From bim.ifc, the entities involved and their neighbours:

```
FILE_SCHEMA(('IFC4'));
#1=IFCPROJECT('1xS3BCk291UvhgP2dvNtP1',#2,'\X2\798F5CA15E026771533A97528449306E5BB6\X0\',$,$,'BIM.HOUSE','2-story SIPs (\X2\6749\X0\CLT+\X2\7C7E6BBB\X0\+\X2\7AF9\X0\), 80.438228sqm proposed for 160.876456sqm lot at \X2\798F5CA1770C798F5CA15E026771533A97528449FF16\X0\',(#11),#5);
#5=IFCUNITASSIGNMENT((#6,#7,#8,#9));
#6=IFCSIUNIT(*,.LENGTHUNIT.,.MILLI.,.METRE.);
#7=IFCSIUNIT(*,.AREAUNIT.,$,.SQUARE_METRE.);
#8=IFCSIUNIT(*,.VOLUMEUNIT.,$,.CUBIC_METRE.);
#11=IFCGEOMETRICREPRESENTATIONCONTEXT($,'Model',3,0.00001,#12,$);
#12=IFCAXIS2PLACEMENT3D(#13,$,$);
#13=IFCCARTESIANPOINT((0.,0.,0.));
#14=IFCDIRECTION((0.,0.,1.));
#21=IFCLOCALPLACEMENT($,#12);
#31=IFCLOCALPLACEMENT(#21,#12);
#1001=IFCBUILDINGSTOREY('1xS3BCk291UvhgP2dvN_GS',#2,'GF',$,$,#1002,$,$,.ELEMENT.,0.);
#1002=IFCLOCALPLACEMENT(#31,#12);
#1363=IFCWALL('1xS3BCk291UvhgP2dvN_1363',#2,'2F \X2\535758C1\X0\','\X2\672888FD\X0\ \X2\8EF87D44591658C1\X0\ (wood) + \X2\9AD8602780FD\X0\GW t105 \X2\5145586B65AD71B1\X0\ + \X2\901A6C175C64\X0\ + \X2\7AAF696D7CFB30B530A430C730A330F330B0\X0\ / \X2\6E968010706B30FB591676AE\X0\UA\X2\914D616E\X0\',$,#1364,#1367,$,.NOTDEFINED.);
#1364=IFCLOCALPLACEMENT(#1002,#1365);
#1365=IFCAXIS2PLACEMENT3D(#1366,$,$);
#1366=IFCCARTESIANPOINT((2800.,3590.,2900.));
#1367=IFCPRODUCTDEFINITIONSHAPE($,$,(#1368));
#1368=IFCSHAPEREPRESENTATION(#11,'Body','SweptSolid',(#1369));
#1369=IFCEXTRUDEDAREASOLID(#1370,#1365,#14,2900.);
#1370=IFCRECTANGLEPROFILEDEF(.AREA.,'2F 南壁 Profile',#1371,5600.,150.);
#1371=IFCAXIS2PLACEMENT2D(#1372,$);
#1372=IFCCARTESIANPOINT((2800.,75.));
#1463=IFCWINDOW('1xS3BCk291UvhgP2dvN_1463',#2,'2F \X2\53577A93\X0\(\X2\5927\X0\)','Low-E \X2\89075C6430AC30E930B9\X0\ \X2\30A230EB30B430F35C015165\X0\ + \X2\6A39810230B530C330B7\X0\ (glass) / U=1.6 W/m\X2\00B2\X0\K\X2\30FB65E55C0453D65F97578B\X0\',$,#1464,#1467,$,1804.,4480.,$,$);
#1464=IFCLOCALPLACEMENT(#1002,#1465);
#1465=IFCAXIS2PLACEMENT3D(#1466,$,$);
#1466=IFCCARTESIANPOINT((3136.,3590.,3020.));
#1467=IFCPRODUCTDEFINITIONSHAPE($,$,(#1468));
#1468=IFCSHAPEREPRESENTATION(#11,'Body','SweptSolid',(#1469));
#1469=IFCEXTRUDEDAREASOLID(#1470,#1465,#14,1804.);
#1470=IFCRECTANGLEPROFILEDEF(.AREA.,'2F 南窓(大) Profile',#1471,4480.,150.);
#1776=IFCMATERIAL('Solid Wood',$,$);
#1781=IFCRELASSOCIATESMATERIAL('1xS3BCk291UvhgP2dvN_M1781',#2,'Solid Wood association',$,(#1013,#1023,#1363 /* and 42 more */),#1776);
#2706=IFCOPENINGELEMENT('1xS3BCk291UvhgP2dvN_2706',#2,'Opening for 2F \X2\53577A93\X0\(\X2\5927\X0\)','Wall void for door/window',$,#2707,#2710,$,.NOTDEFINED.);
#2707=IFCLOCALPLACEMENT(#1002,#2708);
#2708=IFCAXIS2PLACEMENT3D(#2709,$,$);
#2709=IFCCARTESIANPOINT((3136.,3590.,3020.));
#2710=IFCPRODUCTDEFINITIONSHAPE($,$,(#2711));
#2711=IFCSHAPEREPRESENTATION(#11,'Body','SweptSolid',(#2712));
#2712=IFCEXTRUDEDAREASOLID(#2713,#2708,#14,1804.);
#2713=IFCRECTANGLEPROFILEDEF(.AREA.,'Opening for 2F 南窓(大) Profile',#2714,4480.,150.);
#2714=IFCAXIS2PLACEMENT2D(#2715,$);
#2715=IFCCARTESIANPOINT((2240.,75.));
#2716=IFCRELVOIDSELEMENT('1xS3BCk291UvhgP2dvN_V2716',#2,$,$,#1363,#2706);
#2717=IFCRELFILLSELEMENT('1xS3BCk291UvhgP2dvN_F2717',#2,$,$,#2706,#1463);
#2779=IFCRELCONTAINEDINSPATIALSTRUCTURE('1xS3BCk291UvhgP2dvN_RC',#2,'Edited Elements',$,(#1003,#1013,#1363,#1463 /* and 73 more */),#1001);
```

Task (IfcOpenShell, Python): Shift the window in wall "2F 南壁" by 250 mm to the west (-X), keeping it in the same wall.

```python
import ifcopenshell
import ifcopenshell.api.geometry
import ifcopenshell.util.placement
import ifcopenshell.util.unit

model = ifcopenshell.open("bim.ifc")
unit_scale = ifcopenshell.util.unit.calculate_unit_scale(model)

window = model.by_id(1463)
opening = window.FillsVoids[0].RelatingOpeningElement
wall = opening.VoidsElements[0].RelatingBuildingElement

wall_matrix = ifcopenshell.util.placement.get_local_placement(wall.ObjectPlacement)
shift = wall_matrix[:3, 0] * -0.25 / unit_scale
before = ifcopenshell.util.placement.get_local_placement(window.ObjectPlacement)[:3, 3].copy()

# The window is not placed relative to its opening, so move both.
for product in (opening, window):
    matrix = ifcopenshell.util.placement.get_local_placement(product.ObjectPlacement)
    matrix[:3, 3] += shift
    ifcopenshell.api.geometry.edit_object_placement(model, product=product, matrix=matrix, is_si=False)

after = ifcopenshell.util.placement.get_local_placement(window.ObjectPlacement)[:3, 3]
print("window moved by", (after - before).round(3) + 0.0)

model.write("bim_rev.ifc")
```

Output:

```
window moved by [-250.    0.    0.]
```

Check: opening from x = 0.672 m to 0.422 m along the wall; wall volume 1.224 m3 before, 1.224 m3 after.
